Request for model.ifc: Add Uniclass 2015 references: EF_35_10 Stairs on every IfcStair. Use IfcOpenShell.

First a look at what the model holds.

```python
import ifcopenshell

model = ifcopenshell.open("model.ifc")
print(model.schema)
print("classifications:", [c.Name for c in model.by_type("IfcClassification")])
for ifc_class in ("IfcDoor", "IfcRoof", "IfcStair", "IfcWall", "IfcWindow"):
    print(ifc_class, len(model.by_type(ifc_class)))
```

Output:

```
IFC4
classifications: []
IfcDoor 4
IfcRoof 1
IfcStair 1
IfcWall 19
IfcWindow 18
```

```python
import ifcopenshell
import ifcopenshell.api.classification

model = ifcopenshell.open("model.ifc")

system = ifcopenshell.api.classification.add_classification(model, classification="Uniclass 2015")

codes = {
    "IfcStair": ("EF_35_10", "Stairs"),
}
for ifc_class, (code, name) in codes.items():
    products = model.by_type(ifc_class)
    ifcopenshell.api.classification.add_reference(
        model, products=products, classification=system, identification=code, name=name
    )
    print(code, len(products))

model.write("model-out.ifc")
```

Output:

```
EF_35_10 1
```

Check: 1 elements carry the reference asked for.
